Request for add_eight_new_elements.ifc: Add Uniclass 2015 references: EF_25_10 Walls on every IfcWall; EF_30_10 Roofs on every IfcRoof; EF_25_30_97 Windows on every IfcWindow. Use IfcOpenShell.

First a look at what the model holds.

```python
import ifcopenshell

model = ifcopenshell.open("add_eight_new_elements.ifc")
print(model.schema)
print("classifications:", [c.Name for c in model.by_type("IfcClassification")])
for ifc_class in ("IfcDoor", "IfcRoof", "IfcStair", "IfcWall", "IfcWindow"):
    print(ifc_class, len(model.by_type(ifc_class)))
```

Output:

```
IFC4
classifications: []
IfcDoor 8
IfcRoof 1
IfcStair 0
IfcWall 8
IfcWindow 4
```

```python
import ifcopenshell
import ifcopenshell.api.classification

model = ifcopenshell.open("add_eight_new_elements.ifc")

system = ifcopenshell.api.classification.add_classification(model, classification="Uniclass 2015")

codes = {
    "IfcWall": ("EF_25_10", "Walls"),
    "IfcRoof": ("EF_30_10", "Roofs"),
    "IfcWindow": ("EF_25_30_97", "Windows"),
}
for ifc_class, (code, name) in codes.items():
    products = model.by_type(ifc_class)
    ifcopenshell.api.classification.add_reference(
        model, products=products, classification=system, identification=code, name=name
    )
    print(code, len(products))

model.write("add_eight_new_elements_updated.ifc")
```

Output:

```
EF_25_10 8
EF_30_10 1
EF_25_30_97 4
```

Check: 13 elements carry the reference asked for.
